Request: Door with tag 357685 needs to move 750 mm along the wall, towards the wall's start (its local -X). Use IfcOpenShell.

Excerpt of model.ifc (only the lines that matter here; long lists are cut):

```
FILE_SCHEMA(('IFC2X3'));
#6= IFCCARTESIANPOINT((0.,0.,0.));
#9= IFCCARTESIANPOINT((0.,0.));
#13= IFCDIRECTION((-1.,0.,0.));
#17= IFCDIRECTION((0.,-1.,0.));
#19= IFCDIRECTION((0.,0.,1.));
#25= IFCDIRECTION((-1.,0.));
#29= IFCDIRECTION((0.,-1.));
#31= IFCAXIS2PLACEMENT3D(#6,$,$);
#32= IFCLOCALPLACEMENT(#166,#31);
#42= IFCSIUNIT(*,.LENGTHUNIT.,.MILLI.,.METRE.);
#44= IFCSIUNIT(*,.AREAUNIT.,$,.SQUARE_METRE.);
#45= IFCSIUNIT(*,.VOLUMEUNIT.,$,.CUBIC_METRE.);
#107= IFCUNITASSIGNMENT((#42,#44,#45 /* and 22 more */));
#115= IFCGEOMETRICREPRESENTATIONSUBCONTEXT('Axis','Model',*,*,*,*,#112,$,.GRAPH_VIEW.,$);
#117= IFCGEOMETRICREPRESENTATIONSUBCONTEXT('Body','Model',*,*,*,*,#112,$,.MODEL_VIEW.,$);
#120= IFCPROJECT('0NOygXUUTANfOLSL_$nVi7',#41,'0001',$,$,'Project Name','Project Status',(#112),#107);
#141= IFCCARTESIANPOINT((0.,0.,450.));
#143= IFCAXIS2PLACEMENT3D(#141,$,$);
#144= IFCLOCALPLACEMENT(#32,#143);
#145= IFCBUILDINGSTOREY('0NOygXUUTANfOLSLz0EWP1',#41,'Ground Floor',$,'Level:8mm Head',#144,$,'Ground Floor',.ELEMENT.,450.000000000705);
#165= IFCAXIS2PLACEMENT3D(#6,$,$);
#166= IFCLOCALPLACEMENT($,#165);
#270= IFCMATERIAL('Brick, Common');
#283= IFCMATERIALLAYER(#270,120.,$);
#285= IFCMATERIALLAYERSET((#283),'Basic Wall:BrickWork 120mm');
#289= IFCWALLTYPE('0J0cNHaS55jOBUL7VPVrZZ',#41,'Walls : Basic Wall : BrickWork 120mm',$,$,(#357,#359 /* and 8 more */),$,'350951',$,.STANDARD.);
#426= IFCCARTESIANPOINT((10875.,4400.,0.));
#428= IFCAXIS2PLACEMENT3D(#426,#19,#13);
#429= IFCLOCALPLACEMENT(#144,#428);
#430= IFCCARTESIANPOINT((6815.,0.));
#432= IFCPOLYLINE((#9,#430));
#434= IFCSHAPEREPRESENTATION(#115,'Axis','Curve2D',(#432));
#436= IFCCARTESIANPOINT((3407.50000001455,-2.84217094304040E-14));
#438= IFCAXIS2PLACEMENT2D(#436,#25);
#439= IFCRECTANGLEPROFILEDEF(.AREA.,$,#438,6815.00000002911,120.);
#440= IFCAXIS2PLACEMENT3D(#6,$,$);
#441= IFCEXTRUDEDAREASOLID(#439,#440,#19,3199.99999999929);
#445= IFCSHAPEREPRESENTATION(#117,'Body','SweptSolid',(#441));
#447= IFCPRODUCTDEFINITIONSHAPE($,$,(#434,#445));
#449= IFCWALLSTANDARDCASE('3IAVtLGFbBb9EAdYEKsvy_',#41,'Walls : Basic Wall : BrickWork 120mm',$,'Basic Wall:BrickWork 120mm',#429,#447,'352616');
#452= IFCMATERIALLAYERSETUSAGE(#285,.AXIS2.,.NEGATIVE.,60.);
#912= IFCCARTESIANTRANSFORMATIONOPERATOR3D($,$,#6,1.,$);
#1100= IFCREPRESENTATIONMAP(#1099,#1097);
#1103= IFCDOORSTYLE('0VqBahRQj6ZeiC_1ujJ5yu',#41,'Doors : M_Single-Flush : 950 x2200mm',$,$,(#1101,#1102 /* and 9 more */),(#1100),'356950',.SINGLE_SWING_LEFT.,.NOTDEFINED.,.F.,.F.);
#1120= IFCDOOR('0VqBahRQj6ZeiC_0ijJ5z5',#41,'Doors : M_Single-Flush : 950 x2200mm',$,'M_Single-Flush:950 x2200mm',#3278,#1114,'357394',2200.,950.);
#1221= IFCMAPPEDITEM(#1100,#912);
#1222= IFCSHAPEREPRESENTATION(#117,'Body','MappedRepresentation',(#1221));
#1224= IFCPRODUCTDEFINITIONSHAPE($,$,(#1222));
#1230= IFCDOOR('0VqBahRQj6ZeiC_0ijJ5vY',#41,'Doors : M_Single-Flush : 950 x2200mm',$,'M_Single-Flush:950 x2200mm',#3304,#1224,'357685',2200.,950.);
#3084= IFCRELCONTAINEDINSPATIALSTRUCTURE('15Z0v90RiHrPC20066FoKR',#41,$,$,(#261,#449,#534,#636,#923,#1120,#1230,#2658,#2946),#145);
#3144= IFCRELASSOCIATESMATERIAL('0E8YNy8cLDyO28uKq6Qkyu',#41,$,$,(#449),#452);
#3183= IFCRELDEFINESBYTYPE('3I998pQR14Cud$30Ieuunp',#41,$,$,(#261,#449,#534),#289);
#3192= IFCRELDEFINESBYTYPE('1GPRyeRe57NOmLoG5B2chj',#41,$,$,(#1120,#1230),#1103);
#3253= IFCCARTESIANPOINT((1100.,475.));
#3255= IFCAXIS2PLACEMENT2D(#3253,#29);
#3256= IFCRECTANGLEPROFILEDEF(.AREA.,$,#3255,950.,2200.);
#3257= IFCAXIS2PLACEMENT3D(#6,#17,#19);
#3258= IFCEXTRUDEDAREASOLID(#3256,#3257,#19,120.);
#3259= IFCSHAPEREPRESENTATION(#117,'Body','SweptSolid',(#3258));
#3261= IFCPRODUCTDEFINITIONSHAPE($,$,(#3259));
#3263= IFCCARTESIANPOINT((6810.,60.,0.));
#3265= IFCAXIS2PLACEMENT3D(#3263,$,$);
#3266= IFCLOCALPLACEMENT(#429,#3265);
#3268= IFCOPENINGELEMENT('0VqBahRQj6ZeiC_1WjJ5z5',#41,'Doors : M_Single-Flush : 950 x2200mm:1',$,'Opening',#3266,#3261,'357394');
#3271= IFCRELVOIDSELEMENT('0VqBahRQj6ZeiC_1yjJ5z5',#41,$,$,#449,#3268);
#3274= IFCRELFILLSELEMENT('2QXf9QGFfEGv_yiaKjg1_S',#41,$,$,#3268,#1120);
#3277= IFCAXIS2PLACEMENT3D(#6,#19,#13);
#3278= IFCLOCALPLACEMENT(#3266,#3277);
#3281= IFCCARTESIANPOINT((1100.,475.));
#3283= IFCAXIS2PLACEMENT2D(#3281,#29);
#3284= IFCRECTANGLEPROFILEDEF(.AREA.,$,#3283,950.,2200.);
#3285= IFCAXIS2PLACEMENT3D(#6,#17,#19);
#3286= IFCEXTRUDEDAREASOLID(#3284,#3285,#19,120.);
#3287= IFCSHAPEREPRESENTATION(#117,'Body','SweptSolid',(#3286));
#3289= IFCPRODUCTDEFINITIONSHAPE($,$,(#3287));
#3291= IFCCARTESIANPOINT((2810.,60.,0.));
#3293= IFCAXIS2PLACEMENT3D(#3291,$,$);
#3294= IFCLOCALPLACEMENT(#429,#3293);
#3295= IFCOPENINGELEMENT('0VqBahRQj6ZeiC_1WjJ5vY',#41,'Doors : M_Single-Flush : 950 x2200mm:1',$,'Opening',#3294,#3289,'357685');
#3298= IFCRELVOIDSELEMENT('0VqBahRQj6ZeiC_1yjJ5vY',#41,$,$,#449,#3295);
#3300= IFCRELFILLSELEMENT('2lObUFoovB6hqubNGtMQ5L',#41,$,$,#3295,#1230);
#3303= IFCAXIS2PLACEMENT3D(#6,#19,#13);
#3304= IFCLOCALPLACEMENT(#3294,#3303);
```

```python
import ifcopenshell
import ifcopenshell.api.geometry
import ifcopenshell.util.placement
import ifcopenshell.util.unit

model = ifcopenshell.open("model.ifc")
unit_scale = ifcopenshell.util.unit.calculate_unit_scale(model)

door = model.by_guid("0VqBahRQj6ZeiC_0ijJ5vY")
opening = door.FillsVoids[0].RelatingOpeningElement
wall = opening.VoidsElements[0].RelatingBuildingElement

wall_matrix = ifcopenshell.util.placement.get_local_placement(wall.ObjectPlacement)
shift = wall_matrix[:3, 0] * -0.75 / unit_scale
before = ifcopenshell.util.placement.get_local_placement(door.ObjectPlacement)[:3, 3].copy()

# The door is placed relative to its opening, so it follows when the opening moves.
matrix = ifcopenshell.util.placement.get_local_placement(opening.ObjectPlacement)
matrix[:3, 3] += shift
ifcopenshell.api.geometry.edit_object_placement(
    model, product=opening, matrix=matrix, is_si=False, should_transform_children=True
)

after = ifcopenshell.util.placement.get_local_placement(door.ObjectPlacement)[:3, 3]
print("door moved by", (after - before).round(3) + 0.0)

model.write("model-out.ifc")
```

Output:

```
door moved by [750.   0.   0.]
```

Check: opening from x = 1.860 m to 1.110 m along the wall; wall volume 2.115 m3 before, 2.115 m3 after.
